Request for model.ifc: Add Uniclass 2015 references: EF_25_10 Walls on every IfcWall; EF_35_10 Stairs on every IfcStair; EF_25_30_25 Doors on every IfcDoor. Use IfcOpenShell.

First a look at what the model holds.

```python
import ifcopenshell

model = ifcopenshell.open("model.ifc")
print(model.schema)
print("classifications:", [c.Name for c in model.by_type("IfcClassification")])
for ifc_class in ("IfcDoor", "IfcRoof", "IfcStair", "IfcWall", "IfcWindow"):
    print(ifc_class, len(model.by_type(ifc_class)))
```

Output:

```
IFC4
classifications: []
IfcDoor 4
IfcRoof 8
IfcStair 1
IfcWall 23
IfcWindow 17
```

```python
import ifcopenshell
import ifcopenshell.api.classification

model = ifcopenshell.open("model.ifc")

system = ifcopenshell.api.classification.add_classification(model, classification="Uniclass 2015")

codes = {
    "IfcWall": ("EF_25_10", "Walls"),
    "IfcStair": ("EF_35_10", "Stairs"),
    "IfcDoor": ("EF_25_30_25", "Doors"),
}
for ifc_class, (code, name) in codes.items():
    products = model.by_type(ifc_class)
    ifcopenshell.api.classification.add_reference(
        model, products=products, classification=system, identification=code, name=name
    )
    print(code, len(products))

model.write("model_rev.ifc")
```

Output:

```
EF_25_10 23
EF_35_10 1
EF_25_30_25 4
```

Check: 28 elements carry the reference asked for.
